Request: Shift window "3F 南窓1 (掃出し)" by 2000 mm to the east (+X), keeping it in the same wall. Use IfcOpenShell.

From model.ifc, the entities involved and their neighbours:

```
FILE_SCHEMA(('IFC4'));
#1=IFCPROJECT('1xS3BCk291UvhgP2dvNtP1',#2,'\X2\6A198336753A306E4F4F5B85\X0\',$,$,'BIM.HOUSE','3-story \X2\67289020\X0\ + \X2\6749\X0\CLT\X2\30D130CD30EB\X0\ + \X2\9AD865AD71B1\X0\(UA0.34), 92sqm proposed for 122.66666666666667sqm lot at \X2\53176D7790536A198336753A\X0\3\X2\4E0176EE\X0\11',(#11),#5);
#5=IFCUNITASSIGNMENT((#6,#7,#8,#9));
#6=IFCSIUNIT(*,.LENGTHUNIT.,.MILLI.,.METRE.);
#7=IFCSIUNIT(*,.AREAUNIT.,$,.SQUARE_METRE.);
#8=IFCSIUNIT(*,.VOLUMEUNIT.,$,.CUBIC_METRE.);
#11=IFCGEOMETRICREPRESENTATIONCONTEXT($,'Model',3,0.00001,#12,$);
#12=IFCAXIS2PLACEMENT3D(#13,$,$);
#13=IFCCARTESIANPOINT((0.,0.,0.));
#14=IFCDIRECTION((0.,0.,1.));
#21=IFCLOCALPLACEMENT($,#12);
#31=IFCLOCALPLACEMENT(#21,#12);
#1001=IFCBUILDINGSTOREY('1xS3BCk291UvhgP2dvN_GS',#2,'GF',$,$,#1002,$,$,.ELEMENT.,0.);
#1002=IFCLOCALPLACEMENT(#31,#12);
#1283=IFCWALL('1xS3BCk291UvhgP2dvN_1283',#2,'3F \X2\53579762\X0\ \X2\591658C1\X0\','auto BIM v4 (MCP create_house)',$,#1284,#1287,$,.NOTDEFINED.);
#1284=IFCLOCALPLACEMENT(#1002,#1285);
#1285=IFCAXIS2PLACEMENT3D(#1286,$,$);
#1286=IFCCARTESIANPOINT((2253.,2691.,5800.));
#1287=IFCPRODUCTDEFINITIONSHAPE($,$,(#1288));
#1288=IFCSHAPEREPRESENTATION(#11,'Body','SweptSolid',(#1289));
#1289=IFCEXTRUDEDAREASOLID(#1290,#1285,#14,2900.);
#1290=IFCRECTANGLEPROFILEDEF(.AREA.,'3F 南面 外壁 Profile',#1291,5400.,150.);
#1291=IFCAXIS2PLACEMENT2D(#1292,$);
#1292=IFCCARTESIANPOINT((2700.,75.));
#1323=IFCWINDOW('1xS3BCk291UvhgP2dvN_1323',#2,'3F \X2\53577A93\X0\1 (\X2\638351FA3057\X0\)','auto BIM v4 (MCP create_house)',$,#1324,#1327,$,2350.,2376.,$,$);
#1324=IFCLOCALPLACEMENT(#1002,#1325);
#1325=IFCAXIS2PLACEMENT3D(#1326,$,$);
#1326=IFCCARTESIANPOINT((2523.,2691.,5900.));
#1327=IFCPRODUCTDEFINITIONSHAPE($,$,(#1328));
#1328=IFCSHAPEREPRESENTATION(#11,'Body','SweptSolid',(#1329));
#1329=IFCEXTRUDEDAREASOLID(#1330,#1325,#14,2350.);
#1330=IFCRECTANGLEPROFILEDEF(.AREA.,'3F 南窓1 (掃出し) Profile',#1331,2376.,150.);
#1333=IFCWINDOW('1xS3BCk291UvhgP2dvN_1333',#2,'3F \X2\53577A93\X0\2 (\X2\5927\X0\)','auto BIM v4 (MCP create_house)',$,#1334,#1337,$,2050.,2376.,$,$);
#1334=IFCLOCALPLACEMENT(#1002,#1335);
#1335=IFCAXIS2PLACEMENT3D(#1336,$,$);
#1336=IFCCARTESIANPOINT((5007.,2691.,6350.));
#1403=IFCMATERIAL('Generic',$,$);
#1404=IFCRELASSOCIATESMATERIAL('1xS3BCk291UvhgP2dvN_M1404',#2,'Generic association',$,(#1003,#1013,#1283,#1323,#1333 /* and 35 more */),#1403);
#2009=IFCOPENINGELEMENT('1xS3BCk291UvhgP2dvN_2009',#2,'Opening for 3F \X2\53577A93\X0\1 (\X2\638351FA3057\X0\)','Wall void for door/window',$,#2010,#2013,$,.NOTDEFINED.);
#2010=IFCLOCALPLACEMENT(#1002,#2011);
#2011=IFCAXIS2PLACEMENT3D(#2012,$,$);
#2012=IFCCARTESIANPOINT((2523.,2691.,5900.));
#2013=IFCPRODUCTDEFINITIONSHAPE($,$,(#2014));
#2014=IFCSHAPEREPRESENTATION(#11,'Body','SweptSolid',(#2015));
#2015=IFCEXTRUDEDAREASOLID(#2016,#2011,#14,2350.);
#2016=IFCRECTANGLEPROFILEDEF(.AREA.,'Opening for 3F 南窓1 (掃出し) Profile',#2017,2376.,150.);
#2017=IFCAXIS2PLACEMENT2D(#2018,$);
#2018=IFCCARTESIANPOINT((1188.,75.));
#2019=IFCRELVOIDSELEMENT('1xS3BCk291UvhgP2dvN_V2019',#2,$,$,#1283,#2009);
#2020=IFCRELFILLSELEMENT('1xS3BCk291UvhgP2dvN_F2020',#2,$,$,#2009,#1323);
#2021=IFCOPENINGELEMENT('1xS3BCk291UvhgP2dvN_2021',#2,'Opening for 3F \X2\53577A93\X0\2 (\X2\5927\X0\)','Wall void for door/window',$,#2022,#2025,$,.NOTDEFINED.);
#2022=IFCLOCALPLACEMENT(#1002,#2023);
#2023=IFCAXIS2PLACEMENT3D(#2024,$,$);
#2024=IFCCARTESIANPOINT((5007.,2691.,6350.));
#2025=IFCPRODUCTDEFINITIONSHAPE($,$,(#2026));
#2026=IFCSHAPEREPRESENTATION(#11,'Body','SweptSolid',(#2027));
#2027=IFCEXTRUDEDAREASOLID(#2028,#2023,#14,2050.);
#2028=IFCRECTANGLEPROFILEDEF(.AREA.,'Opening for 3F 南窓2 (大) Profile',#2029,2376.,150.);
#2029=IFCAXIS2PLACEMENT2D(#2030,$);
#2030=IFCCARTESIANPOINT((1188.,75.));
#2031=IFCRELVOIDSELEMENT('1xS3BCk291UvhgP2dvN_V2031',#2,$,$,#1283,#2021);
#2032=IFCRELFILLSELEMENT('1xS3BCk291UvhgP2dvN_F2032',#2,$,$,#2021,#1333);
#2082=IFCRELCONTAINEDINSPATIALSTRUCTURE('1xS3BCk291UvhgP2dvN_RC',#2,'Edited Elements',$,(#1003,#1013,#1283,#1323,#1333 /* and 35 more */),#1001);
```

```python
import ifcopenshell
import ifcopenshell.api.geometry
import ifcopenshell.util.placement
import ifcopenshell.util.unit

model = ifcopenshell.open("model.ifc")
unit_scale = ifcopenshell.util.unit.calculate_unit_scale(model)

window = model.by_id(1323)
opening = window.FillsVoids[0].RelatingOpeningElement
wall = opening.VoidsElements[0].RelatingBuildingElement

wall_matrix = ifcopenshell.util.placement.get_local_placement(wall.ObjectPlacement)
shift = wall_matrix[:3, 0] * 2 / unit_scale
before = ifcopenshell.util.placement.get_local_placement(window.ObjectPlacement)[:3, 3].copy()

# The window is not placed relative to its opening, so move both.
for product in (opening, window):
    matrix = ifcopenshell.util.placement.get_local_placement(product.ObjectPlacement)
    matrix[:3, 3] += shift
    ifcopenshell.api.geometry.edit_object_placement(model, product=product, matrix=matrix, is_si=False)

after = ifcopenshell.util.placement.get_local_placement(window.ObjectPlacement)[:3, 3]
print("window moved by", (after - before).round(3) + 0.0)

model.write("model-out.ifc")
```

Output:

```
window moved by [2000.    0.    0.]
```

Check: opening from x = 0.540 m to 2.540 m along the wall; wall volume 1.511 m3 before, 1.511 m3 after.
